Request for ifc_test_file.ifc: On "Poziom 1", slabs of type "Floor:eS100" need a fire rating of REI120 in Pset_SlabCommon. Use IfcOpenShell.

First a look at what the model holds.

```python
import ifcopenshell
import ifcopenshell.util.element

model = ifcopenshell.open("ifc_test_file.ifc")
print(model.schema)
storey = next(s for s in model.by_type("IfcBuildingStorey") if s.Name == "Poziom 1")
slabs = [e for e in ifcopenshell.util.element.get_decomposition(storey) if e.is_a("IfcSlab")]
seen = {}
for e in slabs:
    element_type = ifcopenshell.util.element.get_type(e)
    key = (element_type.Name if element_type != e and element_type else None, ifcopenshell.util.element.get_pset(e, "Pset_SlabCommon", "FireRating"))
    seen[key] = seen.get(key, 0) + 1
for (name, value), count in sorted(seen.items(), key=str):
    print(count, "x", name, "|", value)
```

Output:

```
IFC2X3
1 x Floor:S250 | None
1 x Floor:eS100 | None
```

```python
import ifcopenshell
import ifcopenshell.api.pset
import ifcopenshell.util.element

model = ifcopenshell.open("ifc_test_file.ifc")

storey = next(s for s in model.by_type("IfcBuildingStorey") if s.Name == "Poziom 1")
slabs = [e for e in ifcopenshell.util.element.get_decomposition(storey) if e.is_a("IfcSlab")]

count = 0
for e in slabs:
    element_type = ifcopenshell.util.element.get_type(e)
    if element_type in (None, e) or element_type.Name != "Floor:eS100":
        continue
    # add_pset returns the element's existing set when there is one.
    pset = ifcopenshell.api.pset.add_pset(model, product=e, name="Pset_SlabCommon")
    ifcopenshell.api.pset.edit_pset(model, pset=pset, properties={"FireRating": "REI120"})
    count += 1

print(count, "slabs updated")

model.write("ifc_test_file-out.ifc")
```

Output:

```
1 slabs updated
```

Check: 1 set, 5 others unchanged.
